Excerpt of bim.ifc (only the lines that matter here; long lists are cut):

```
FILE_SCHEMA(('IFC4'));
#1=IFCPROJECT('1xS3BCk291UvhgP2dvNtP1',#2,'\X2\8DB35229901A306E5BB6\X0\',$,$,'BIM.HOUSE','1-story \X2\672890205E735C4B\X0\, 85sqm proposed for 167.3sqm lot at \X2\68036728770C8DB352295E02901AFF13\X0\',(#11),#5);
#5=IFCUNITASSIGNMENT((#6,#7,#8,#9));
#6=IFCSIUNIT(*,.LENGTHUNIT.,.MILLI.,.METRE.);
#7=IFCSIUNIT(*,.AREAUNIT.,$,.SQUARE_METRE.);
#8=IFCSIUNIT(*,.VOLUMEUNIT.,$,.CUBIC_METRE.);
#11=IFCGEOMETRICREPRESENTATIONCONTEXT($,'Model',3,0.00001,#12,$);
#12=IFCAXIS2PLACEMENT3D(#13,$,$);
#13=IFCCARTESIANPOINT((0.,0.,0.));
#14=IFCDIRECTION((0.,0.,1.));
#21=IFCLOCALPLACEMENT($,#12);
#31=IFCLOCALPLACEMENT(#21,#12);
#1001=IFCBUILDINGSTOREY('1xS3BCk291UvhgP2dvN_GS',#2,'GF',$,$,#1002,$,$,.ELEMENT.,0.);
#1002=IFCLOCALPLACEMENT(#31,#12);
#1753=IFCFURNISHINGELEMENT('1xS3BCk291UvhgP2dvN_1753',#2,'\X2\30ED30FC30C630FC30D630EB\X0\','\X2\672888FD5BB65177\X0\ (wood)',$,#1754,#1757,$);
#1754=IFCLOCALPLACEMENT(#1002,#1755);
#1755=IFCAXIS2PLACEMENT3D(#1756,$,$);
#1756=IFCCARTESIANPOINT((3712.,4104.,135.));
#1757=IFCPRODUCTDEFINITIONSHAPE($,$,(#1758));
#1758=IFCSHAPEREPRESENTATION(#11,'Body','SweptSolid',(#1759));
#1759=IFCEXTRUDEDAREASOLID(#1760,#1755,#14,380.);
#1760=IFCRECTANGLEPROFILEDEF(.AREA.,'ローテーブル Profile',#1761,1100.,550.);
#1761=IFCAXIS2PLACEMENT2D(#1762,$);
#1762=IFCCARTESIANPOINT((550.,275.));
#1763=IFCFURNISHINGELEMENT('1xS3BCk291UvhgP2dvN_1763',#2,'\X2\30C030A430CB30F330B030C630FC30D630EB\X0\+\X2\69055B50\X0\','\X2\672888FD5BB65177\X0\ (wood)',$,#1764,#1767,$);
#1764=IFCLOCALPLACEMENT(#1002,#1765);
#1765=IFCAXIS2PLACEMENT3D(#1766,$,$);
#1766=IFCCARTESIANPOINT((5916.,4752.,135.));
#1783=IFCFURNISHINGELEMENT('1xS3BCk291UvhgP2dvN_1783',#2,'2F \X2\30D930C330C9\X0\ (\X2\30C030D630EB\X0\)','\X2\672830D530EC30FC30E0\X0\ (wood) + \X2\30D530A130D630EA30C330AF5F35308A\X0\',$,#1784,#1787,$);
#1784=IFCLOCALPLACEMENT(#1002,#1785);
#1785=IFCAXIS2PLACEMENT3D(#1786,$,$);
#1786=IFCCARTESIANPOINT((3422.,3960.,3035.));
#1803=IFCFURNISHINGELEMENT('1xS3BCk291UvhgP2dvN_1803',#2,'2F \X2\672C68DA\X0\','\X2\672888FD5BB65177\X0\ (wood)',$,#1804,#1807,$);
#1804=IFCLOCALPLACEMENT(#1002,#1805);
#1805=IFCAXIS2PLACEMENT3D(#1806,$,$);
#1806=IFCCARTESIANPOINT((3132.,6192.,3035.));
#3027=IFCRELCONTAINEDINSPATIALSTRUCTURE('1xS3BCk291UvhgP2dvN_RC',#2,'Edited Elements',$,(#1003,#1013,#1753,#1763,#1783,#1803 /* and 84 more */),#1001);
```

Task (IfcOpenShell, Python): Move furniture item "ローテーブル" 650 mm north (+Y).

```python
import ifcopenshell
import ifcopenshell.api.geometry
import ifcopenshell.util.placement

model = ifcopenshell.open("bim.ifc")

item = model.by_guid("1xS3BCk291UvhgP2dvN_1753")
matrix = ifcopenshell.util.placement.get_local_placement(item.ObjectPlacement)
matrix[1, 3] += 650.0
ifcopenshell.api.geometry.edit_object_placement(model, product=item, matrix=matrix, is_si=False)

print(ifcopenshell.util.placement.get_local_placement(item.ObjectPlacement).round(3) + 0.0)

model.write("bim_edited.ifc")
```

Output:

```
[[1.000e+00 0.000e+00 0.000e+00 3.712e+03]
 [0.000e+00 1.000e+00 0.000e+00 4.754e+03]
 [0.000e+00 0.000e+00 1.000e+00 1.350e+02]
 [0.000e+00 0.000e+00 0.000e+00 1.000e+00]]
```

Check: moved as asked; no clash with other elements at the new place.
